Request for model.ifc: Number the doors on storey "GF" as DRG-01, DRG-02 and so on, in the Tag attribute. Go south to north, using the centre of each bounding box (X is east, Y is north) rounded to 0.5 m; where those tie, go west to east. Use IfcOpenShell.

First a look at what the model holds.

```python
import ifcopenshell
import ifcopenshell.util.element
import ifcopenshell.util.placement

model = ifcopenshell.open("model.ifc")
print(model.schema)
storey = next(s for s in model.by_type("IfcBuildingStorey") if s.Name == "GF")
doors = [e for e in ifcopenshell.util.element.get_decomposition(storey) if e.is_a("IfcDoor")]
for e in sorted(doors, key=lambda e: e.id()):
    origin = ifcopenshell.util.placement.get_local_placement(e.ObjectPlacement)[:3, 3]
    print(e.id(), e.Tag, e.Name, origin.round(2) + 0.0, sep=" | ")
```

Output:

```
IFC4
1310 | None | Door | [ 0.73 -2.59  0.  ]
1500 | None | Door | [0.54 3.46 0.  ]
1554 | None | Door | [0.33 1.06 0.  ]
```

```python
import ifcopenshell
import ifcopenshell.geom
import ifcopenshell.util.element
import ifcopenshell.util.shape

model = ifcopenshell.open("model.ifc")
settings = ifcopenshell.geom.settings()
settings.set("use-world-coords", True)


def centre(element):
    shape = ifcopenshell.geom.create_shape(settings, element)
    return ifcopenshell.util.shape.get_bbox_centroid(shape.geometry)


storey = next(s for s in model.by_type("IfcBuildingStorey") if s.Name == "GF")
doors = [e for e in ifcopenshell.util.element.get_decomposition(storey) if e.is_a("IfcDoor")]

# Insertion points can sit at a corner or the storey origin, so sort by the geometry (in metres).
centres = {e: centre(e) for e in doors}
doors.sort(key=lambda e: (round(centres[e][1] / 0.5), centres[e][0]))

for i, e in enumerate(doors, start=1):
    number = f"DRG-{i:02d}"
    e.Tag = number
    print(e.id(), number)

model.write("model_v2.ifc")
```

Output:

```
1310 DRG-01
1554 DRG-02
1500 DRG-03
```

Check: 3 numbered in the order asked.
